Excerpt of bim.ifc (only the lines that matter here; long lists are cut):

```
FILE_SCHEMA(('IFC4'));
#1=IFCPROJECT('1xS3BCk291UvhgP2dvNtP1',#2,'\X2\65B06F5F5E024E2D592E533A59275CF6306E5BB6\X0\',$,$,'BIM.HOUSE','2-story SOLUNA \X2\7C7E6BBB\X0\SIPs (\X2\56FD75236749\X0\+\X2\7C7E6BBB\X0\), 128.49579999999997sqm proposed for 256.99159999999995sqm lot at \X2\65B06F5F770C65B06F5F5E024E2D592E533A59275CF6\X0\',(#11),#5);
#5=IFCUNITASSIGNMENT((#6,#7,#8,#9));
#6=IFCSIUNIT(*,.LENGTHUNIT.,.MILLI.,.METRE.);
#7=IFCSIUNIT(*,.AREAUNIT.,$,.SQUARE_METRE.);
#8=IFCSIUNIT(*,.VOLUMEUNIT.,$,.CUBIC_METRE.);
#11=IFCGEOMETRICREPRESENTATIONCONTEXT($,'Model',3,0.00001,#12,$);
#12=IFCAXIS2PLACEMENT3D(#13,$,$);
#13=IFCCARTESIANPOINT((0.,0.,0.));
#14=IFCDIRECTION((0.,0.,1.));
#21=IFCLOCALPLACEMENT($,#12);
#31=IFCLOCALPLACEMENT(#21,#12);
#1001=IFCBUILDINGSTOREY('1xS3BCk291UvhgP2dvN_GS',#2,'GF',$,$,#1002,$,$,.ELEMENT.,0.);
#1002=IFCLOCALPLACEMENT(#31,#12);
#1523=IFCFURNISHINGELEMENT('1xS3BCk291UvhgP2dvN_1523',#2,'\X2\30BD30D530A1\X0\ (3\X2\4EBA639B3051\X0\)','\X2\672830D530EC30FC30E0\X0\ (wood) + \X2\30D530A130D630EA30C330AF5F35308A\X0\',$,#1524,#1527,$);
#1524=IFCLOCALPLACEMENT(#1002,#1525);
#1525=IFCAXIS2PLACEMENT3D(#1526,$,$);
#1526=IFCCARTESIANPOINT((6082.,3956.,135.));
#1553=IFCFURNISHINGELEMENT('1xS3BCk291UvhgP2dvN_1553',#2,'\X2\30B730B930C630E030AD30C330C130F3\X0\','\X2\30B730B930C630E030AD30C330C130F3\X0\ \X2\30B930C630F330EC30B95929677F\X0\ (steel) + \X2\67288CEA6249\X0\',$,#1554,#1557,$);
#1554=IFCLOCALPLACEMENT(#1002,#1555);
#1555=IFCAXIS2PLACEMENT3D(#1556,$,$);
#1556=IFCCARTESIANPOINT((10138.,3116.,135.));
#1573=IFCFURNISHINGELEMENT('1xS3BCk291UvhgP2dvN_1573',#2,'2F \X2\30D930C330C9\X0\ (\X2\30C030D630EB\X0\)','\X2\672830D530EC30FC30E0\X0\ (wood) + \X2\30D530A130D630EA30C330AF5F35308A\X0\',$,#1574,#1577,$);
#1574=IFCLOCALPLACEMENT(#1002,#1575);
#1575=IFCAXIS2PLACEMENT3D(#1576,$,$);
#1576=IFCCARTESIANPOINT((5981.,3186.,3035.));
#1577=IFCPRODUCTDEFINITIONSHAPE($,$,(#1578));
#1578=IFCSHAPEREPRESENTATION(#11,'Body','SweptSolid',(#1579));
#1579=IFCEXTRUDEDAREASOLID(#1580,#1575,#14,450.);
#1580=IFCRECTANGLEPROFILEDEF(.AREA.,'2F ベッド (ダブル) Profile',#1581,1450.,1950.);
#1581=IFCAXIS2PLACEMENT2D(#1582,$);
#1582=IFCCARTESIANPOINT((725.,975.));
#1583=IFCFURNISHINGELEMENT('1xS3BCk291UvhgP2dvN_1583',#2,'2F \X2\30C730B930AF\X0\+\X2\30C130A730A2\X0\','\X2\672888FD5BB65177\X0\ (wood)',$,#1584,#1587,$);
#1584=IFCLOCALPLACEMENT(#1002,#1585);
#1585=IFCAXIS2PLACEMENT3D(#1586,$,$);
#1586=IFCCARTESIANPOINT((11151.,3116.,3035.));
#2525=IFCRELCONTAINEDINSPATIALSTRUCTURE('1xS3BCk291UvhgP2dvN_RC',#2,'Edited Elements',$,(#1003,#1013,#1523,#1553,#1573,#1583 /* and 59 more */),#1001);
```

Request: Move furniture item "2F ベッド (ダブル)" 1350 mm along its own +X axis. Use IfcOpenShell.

```python
import ifcopenshell
import ifcopenshell.api.geometry
import ifcopenshell.util.placement
import ifcopenshell.util.unit

model = ifcopenshell.open("bim.ifc")
unit_scale = ifcopenshell.util.unit.calculate_unit_scale(model)

item = model.by_id(1573)
matrix = ifcopenshell.util.placement.get_local_placement(item.ObjectPlacement)
matrix[:3, 3] += matrix[:3, 0] * 1.35 / unit_scale
ifcopenshell.api.geometry.edit_object_placement(model, product=item, matrix=matrix, is_si=False)

print(ifcopenshell.util.placement.get_local_placement(item.ObjectPlacement).round(3) + 0.0)

model.write("bim-out.ifc")
```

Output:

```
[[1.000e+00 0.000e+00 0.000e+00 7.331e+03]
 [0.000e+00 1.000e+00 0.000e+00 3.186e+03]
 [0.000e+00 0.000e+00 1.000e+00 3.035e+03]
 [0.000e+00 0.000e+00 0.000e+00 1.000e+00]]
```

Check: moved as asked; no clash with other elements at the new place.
